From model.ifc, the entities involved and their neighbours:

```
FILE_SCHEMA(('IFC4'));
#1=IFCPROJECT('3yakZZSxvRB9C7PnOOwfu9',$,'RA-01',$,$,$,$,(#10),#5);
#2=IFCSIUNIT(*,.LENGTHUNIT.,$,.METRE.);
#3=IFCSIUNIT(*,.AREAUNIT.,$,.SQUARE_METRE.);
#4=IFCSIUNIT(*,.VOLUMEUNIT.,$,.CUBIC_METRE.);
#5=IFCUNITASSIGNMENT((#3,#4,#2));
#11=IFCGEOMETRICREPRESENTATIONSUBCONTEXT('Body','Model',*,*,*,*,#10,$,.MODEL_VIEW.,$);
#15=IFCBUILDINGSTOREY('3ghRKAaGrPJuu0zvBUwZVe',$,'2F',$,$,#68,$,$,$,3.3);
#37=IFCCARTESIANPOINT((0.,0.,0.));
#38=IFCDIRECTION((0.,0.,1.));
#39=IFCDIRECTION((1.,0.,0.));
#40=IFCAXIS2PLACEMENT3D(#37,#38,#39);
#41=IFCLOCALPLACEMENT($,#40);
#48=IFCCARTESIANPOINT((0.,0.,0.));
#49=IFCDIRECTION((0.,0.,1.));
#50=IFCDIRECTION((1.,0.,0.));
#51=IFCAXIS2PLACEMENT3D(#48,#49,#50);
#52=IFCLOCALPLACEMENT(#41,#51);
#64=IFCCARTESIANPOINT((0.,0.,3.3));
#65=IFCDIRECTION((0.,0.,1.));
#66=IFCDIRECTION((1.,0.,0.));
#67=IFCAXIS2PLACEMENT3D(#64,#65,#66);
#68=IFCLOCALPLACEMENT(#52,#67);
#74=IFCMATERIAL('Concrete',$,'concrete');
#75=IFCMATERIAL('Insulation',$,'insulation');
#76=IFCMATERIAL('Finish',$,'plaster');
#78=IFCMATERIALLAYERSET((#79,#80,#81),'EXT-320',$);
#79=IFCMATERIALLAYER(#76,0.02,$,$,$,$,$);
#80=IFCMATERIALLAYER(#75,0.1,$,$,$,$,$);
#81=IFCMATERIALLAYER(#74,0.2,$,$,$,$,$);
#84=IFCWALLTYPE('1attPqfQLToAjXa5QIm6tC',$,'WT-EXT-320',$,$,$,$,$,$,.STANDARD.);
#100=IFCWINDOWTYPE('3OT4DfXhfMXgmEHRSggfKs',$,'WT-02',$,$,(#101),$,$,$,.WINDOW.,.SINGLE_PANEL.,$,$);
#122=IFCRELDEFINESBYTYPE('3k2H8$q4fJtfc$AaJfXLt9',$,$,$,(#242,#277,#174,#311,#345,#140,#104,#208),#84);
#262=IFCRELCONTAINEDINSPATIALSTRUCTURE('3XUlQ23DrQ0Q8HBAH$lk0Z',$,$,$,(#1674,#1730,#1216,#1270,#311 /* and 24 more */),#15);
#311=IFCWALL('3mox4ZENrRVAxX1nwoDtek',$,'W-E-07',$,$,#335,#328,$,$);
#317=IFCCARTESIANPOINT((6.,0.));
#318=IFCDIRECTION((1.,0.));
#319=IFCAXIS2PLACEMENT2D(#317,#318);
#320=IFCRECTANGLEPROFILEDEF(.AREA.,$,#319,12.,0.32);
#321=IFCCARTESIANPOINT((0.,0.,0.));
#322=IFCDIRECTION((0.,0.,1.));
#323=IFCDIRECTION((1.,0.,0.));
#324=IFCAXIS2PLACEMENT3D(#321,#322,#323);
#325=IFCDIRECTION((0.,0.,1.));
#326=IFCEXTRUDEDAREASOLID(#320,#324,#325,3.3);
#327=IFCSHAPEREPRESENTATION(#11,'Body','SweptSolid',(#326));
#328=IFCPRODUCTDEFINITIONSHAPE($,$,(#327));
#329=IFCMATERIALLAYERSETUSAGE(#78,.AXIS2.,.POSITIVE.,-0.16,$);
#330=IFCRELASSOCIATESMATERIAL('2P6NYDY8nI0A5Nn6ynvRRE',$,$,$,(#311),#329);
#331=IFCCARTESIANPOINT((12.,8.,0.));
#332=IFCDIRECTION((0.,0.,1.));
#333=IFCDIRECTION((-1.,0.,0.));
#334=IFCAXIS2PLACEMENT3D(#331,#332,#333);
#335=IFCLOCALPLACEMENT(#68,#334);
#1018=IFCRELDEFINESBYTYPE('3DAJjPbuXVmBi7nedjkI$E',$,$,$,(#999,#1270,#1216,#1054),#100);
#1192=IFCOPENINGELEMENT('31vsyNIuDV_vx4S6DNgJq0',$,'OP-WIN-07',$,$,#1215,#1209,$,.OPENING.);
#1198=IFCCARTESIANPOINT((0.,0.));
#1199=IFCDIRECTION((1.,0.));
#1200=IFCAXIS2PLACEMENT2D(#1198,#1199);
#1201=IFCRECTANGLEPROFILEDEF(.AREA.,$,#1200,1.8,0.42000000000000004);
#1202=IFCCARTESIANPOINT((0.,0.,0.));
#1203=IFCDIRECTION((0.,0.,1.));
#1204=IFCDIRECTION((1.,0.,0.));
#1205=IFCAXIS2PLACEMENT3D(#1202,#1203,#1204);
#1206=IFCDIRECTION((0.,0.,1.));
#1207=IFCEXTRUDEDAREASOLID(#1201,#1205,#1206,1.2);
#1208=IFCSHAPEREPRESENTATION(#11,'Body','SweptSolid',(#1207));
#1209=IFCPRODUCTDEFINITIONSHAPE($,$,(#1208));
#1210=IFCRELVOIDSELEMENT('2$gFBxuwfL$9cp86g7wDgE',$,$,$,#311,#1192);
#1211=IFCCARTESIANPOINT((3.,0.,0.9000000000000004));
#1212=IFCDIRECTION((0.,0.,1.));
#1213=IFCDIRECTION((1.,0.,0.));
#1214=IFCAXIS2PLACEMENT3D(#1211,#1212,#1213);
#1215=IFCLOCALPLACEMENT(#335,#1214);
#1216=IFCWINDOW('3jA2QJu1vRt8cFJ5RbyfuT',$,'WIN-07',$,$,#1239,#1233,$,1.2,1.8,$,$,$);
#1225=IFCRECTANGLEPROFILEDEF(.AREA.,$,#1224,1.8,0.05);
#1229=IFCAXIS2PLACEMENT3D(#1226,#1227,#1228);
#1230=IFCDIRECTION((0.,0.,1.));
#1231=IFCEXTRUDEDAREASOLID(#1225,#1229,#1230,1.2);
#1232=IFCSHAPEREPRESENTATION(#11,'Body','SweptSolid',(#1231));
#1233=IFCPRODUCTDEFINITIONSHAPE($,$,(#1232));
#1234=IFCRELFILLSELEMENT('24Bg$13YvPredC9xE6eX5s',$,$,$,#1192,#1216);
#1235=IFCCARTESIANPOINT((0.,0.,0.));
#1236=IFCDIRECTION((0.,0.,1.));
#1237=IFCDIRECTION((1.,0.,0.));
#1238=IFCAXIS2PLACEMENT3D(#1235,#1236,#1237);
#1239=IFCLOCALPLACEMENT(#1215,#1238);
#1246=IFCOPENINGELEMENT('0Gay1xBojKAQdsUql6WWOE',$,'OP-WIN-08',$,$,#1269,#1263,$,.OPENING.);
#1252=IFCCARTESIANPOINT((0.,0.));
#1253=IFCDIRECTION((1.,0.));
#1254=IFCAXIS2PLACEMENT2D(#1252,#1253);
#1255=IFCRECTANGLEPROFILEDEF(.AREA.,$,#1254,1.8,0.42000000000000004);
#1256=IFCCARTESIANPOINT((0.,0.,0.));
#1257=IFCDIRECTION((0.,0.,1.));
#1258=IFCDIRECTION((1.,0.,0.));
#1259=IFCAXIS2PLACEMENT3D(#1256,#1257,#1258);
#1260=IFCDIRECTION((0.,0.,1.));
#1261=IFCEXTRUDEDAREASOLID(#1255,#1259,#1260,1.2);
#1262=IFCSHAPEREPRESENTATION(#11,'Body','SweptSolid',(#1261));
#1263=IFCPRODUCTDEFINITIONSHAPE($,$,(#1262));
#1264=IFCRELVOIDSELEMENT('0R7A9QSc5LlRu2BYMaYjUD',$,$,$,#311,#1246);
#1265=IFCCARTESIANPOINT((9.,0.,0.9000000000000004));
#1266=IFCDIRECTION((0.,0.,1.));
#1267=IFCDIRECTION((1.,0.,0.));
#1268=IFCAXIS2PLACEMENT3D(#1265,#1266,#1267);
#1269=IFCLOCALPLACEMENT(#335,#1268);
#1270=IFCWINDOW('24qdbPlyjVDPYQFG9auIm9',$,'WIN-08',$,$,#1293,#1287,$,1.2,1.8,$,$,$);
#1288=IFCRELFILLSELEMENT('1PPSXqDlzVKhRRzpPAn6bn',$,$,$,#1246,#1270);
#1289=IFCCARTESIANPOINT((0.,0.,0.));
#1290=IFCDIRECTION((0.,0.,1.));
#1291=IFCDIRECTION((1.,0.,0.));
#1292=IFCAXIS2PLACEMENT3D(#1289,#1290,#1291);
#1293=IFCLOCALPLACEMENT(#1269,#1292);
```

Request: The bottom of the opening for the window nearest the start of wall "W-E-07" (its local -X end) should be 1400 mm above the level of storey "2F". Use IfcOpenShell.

```python
import numpy as np
import ifcopenshell
import ifcopenshell.api.geometry
import ifcopenshell.geom
import ifcopenshell.util.element
import ifcopenshell.util.placement
import ifcopenshell.util.shape
import ifcopenshell.util.unit

model = ifcopenshell.open("model.ifc")
unit_scale = ifcopenshell.util.unit.calculate_unit_scale(model)

window = model.by_id(1216)
opening = window.FillsVoids[0].RelatingOpeningElement
storey = ifcopenshell.util.element.get_container(window, ifc_class="IfcBuildingStorey")
level = ifcopenshell.util.placement.get_local_placement(storey.ObjectPlacement)[2, 3]

# The opening's origin need not be at the sill, so measure its lowest point.
shape = ifcopenshell.geom.create_shape(ifcopenshell.geom.settings(), opening)
bottom = ifcopenshell.util.shape.get_shape_bottom_elevation(shape, shape.geometry) / unit_scale
dz = level + 1.4 / unit_scale - bottom

shift = np.array([0.0, 0.0, dz])
# The window is placed relative to its opening, so it follows when the opening moves.
matrix = ifcopenshell.util.placement.get_local_placement(opening.ObjectPlacement)
matrix[:3, 3] += shift
ifcopenshell.api.geometry.edit_object_placement(
    model, product=opening, matrix=matrix, is_si=False, should_transform_children=True
)

print(f"moved by {dz * unit_scale:+.3f} m")

model.write("model_rev.ifc")
```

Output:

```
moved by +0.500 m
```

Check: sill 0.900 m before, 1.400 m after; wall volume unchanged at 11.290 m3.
